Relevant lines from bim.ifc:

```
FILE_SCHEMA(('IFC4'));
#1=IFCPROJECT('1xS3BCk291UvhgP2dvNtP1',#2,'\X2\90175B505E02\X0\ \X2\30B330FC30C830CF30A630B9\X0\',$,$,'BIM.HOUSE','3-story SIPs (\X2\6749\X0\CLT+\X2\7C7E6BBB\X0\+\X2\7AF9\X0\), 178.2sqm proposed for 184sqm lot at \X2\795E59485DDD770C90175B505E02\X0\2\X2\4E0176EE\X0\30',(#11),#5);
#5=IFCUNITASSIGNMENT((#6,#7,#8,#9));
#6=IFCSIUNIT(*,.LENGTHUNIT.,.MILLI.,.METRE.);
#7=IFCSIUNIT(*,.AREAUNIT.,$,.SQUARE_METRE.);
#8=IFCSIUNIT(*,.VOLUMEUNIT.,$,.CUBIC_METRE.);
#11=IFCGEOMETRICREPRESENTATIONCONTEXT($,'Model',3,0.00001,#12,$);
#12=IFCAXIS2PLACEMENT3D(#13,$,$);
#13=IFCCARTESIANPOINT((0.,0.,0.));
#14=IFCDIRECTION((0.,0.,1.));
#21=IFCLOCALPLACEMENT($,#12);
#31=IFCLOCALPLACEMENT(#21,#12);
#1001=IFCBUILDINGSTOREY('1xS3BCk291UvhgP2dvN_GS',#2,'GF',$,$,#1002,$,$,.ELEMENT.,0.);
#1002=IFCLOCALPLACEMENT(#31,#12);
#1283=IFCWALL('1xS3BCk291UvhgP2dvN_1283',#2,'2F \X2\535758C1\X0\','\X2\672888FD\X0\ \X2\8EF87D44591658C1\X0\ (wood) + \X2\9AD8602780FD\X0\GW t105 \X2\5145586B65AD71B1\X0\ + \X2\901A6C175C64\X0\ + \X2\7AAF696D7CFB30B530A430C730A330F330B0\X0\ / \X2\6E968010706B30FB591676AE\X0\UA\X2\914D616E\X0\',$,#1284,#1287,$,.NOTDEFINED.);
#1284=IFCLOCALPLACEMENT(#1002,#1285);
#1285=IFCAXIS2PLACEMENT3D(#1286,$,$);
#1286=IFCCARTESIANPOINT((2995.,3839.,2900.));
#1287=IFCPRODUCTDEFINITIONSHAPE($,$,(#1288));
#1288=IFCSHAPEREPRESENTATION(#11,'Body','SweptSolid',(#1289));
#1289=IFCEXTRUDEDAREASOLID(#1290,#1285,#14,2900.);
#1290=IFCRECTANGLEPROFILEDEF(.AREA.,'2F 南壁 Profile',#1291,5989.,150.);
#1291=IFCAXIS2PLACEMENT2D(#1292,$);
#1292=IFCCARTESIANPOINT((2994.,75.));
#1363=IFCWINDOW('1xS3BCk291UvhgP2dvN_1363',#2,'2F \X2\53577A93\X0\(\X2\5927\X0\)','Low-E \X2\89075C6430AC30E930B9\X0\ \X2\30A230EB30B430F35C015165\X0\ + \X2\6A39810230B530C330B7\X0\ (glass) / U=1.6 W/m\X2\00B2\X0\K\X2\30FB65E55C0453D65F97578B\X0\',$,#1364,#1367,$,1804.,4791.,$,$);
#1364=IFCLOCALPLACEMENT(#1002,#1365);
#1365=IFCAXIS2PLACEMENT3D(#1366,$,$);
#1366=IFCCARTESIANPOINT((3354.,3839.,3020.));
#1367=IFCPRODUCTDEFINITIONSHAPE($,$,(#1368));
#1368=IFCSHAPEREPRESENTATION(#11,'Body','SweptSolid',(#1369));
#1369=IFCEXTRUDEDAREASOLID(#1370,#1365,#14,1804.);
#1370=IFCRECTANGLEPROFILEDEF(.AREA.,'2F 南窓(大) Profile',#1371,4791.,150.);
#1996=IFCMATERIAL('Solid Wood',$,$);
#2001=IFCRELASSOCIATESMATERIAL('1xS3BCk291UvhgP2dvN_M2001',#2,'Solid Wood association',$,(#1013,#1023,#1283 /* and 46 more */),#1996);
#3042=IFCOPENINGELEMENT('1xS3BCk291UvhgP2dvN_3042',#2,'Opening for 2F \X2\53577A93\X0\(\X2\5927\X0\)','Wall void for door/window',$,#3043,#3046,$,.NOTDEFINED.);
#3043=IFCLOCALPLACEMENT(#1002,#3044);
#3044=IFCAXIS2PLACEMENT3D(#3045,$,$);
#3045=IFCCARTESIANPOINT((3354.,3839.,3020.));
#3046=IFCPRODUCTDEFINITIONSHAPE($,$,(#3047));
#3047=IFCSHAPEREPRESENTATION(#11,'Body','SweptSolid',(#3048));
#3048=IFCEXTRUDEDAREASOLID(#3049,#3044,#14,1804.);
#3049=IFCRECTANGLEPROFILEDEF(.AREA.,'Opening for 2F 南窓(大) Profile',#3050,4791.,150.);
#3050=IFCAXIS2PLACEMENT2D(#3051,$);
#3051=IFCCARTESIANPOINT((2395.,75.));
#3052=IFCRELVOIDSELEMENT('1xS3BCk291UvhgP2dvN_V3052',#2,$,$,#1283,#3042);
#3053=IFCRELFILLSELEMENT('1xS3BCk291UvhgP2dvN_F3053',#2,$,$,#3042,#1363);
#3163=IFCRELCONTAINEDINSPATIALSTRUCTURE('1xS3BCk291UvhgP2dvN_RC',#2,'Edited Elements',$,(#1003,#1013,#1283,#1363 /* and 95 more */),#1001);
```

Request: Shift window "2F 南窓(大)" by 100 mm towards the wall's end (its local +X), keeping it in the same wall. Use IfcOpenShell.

```python
import ifcopenshell
import ifcopenshell.api.geometry
import ifcopenshell.util.placement

model = ifcopenshell.open("bim.ifc")

window = model.by_id(1363)
opening = window.FillsVoids[0].RelatingOpeningElement
wall = opening.VoidsElements[0].RelatingBuildingElement

wall_matrix = ifcopenshell.util.placement.get_local_placement(wall.ObjectPlacement)
shift = wall_matrix[:3, 0] * 100.0
before = ifcopenshell.util.placement.get_local_placement(window.ObjectPlacement)[:3, 3].copy()

# The window is not placed relative to its opening, so move both.
for product in (opening, window):
    matrix = ifcopenshell.util.placement.get_local_placement(product.ObjectPlacement)
    matrix[:3, 3] += shift
    ifcopenshell.api.geometry.edit_object_placement(model, product=product, matrix=matrix, is_si=False)

after = ifcopenshell.util.placement.get_local_placement(window.ObjectPlacement)[:3, 3]
print("window moved by", (after - before).round(3) + 0.0)

model.write("bim_updated.ifc")
```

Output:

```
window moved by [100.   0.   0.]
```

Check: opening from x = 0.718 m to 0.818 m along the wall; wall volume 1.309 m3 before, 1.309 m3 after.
